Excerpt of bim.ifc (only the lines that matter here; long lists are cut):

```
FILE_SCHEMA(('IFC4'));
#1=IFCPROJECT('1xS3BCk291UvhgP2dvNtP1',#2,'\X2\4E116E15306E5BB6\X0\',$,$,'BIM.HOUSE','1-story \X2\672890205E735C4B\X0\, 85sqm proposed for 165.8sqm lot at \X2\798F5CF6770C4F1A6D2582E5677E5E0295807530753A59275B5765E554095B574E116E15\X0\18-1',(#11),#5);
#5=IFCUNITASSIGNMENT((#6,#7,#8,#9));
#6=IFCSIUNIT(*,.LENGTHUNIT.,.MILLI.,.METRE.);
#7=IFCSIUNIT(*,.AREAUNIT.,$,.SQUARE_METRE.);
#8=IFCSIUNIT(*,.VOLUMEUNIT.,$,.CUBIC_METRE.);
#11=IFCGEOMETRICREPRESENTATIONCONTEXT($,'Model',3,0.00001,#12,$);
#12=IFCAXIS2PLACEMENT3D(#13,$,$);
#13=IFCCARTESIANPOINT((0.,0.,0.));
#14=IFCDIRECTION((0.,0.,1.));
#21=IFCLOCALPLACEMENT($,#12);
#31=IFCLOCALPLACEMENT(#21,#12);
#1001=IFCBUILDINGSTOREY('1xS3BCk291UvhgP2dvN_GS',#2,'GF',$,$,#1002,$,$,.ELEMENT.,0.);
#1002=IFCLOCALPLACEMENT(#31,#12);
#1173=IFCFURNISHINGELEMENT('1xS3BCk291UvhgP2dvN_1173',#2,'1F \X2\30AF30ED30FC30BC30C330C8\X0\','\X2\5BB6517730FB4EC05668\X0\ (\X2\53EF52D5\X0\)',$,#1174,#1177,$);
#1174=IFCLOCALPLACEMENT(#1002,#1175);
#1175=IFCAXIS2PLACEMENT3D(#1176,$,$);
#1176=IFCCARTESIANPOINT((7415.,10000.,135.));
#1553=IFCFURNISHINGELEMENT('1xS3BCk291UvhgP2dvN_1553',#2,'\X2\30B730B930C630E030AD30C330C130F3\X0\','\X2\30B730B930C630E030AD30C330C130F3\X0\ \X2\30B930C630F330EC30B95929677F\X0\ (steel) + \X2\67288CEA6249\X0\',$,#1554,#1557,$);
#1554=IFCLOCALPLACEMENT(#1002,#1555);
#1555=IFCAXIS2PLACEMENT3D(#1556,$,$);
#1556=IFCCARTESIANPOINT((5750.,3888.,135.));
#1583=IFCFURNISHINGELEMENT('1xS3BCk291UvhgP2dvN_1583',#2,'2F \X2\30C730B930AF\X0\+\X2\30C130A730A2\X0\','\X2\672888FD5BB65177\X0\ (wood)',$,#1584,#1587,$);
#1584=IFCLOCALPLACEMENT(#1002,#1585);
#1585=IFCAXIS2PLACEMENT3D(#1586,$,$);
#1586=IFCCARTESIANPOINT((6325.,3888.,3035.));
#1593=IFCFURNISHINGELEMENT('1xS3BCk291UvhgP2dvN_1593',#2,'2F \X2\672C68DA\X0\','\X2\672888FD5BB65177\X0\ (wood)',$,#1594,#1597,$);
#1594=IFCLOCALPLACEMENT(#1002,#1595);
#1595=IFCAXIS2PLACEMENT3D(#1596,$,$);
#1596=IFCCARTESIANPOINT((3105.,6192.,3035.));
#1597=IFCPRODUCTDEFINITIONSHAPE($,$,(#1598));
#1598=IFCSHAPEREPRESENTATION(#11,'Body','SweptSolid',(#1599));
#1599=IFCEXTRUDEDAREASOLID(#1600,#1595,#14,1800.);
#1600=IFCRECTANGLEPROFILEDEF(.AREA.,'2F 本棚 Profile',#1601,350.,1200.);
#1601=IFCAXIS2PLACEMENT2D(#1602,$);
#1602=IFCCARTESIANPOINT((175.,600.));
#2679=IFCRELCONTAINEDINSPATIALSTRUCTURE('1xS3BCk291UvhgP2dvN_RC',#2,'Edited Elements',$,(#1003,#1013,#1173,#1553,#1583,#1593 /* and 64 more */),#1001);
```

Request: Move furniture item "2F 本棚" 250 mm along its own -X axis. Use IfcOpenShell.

```python
import ifcopenshell
import ifcopenshell.api.geometry
import ifcopenshell.util.placement
import ifcopenshell.util.unit

model = ifcopenshell.open("bim.ifc")
unit_scale = ifcopenshell.util.unit.calculate_unit_scale(model)

item = model.by_guid("1xS3BCk291UvhgP2dvN_1593")
matrix = ifcopenshell.util.placement.get_local_placement(item.ObjectPlacement)
matrix[:3, 3] -= matrix[:3, 0] * 0.25 / unit_scale
ifcopenshell.api.geometry.edit_object_placement(model, product=item, matrix=matrix, is_si=False)

print(ifcopenshell.util.placement.get_local_placement(item.ObjectPlacement).round(3) + 0.0)

model.write("bim_rev.ifc")
```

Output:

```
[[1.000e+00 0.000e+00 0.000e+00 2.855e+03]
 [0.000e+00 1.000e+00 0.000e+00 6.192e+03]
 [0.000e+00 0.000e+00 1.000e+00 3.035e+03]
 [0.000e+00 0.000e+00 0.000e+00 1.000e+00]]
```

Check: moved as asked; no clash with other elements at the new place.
